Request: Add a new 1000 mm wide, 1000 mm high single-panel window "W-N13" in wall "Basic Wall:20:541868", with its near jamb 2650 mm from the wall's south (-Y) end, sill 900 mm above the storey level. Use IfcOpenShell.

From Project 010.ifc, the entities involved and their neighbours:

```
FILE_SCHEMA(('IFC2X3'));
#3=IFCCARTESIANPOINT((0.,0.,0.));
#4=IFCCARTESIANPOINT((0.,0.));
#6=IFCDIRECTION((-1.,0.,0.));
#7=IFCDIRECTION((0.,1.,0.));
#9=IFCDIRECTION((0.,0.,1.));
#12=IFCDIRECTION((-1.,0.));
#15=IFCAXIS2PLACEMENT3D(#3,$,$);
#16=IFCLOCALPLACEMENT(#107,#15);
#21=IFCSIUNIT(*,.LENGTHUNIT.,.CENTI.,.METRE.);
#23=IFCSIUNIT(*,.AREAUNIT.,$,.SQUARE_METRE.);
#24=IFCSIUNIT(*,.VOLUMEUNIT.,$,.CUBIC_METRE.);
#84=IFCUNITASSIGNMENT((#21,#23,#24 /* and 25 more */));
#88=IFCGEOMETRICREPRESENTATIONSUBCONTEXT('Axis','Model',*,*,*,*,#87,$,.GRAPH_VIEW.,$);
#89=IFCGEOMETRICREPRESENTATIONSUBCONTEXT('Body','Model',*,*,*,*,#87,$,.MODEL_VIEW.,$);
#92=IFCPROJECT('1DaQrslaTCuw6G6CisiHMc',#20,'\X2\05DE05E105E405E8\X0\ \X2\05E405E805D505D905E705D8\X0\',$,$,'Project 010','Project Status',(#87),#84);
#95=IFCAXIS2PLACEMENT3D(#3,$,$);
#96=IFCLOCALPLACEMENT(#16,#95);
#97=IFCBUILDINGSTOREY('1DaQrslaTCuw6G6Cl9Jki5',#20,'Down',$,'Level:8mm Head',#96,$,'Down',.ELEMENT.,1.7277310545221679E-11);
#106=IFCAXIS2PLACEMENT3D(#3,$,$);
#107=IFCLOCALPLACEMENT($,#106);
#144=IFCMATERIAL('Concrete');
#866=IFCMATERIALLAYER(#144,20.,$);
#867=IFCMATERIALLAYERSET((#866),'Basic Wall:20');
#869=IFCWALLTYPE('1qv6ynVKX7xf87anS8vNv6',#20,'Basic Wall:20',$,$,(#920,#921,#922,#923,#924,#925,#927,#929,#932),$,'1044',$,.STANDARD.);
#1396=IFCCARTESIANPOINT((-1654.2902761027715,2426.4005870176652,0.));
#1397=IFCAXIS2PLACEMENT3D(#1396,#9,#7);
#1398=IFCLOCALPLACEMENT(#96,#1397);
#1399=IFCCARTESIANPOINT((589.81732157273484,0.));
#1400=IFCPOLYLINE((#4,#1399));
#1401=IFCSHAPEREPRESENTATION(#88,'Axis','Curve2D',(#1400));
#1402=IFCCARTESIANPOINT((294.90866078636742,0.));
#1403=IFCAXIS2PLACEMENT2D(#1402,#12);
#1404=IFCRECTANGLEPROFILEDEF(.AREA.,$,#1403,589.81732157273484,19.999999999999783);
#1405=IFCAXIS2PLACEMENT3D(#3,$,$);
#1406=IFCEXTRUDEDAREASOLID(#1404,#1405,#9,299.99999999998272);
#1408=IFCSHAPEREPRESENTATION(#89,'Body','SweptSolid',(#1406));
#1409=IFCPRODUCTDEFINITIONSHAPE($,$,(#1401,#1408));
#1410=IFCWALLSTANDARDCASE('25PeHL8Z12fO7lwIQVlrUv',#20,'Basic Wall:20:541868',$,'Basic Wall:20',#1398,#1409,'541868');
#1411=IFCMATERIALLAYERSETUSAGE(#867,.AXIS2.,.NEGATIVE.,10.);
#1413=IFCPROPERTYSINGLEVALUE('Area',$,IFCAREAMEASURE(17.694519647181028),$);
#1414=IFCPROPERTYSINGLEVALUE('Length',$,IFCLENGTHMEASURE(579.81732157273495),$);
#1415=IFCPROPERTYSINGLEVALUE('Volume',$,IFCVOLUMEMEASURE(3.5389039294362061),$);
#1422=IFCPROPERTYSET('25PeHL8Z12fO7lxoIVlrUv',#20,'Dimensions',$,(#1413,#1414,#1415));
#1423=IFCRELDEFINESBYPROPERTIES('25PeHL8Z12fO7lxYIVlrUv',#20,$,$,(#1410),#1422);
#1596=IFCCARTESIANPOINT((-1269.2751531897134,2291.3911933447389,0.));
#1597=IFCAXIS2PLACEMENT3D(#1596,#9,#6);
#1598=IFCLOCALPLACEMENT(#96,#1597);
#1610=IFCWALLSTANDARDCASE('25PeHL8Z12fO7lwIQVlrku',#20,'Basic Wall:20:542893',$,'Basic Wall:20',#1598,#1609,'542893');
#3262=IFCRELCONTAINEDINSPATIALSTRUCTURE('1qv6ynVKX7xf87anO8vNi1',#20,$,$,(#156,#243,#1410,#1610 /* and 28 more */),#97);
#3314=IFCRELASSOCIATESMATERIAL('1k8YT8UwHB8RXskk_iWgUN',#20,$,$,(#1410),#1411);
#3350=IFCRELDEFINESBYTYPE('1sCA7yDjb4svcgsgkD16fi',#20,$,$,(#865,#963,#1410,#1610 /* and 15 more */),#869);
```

```python
import numpy as np
import ifcopenshell
import ifcopenshell.api.feature
import ifcopenshell.api.geometry
import ifcopenshell.api.pset
import ifcopenshell.api.root
import ifcopenshell.api.spatial
import ifcopenshell.api.type
import ifcopenshell.geom
import ifcopenshell.util.element
import ifcopenshell.util.placement
import ifcopenshell.util.representation
import ifcopenshell.util.shape
import ifcopenshell.util.unit

model = ifcopenshell.open("Project 010.ifc")
unit_scale = ifcopenshell.util.unit.calculate_unit_scale(model)
area_scale = ifcopenshell.util.unit.calculate_unit_scale(model, "AREAUNIT")
volume_scale = ifcopenshell.util.unit.calculate_unit_scale(model, "VOLUMEUNIT")
settings = ifcopenshell.geom.settings()


def volume(element):
    """Net volume in cubic metres, openings subtracted."""
    shape = ifcopenshell.geom.create_shape(settings, element)
    return ifcopenshell.util.shape.get_volume(shape.geometry)


wall = model.by_id(1410)
storey = ifcopenshell.util.element.get_container(wall, ifc_class="IfcBuildingStorey")
context = ifcopenshell.util.representation.get_context(model, "Model", "Body", "MODEL_VIEW")
before = volume(wall)

width, height, from_end, sill = 1, 1, 2.65, 0.9  # metres

# The wall runs along its own X axis, and the end named is its -X end.
wall_shape = ifcopenshell.geom.create_shape(settings, wall)
x, y, z = ifcopenshell.util.shape.get_vertices(wall_shape.geometry).T
start = x.min() + from_end
face, thickness = float(y.min()), float(y.max() - y.min())
wall_matrix = ifcopenshell.util.placement.get_local_placement(wall.ObjectPlacement)
level = ifcopenshell.util.placement.get_local_placement(storey.ObjectPlacement)[2, 3]


def in_wall(x, y):
    """Placement at x, y metres in the wall's axes, at sill height."""
    matrix = wall_matrix.copy()
    matrix[:, 3] = wall_matrix @ np.array([x / unit_scale, y / unit_scale, 0.0, 1.0])
    matrix[2, 3] = level + sill / unit_scale
    return matrix


# Opening: a box that overshoots both wall faces by 50 mm.
opening = ifcopenshell.api.root.create_entity(model, ifc_class="IfcOpeningElement")
box = ifcopenshell.api.geometry.add_wall_representation(
    model, context=context, length=width, height=height, thickness=thickness + 0.1
)
ifcopenshell.api.geometry.assign_representation(model, product=opening, representation=box)
ifcopenshell.api.geometry.edit_object_placement(model, product=opening, matrix=in_wall(start, face - 0.05), is_si=False)
ifcopenshell.api.feature.add_feature(model, feature=opening, element=wall)

window = ifcopenshell.api.root.create_entity(model, ifc_class="IfcWindow", name="W-N13")
window.OverallWidth, window.OverallHeight = width / unit_scale, height / unit_scale
body = ifcopenshell.api.geometry.add_window_representation(
    model,
    context=context,
    overall_width=window.OverallWidth,
    overall_height=window.OverallHeight,
    partition_type="SINGLE_PANEL",
)
ifcopenshell.api.geometry.assign_representation(model, product=window, representation=body)
ifcopenshell.api.spatial.assign_container(model, products=[window], relating_structure=storey)
fills = ifcopenshell.api.feature.add_filling(model, opening=opening, element=window)
fills.OwnerHistory = window.OwnerHistory  # required in IFC2X3

# IFC2X3 keeps the operation on the window style.
style = ifcopenshell.api.root.create_entity(model, ifc_class="IfcWindowStyle", name="W-N13")
style.OperationType, style.ConstructionType = "SINGLE_PANEL", "NOTDEFINED"
style.ParameterTakesPrecedence = style.Sizeable = False
ifcopenshell.api.type.assign_type(model, related_objects=[window], relating_type=style)

# Centre the window in the wall's thickness.
ifcopenshell.api.geometry.edit_object_placement(model, product=window, matrix=in_wall(start, face), is_si=False)
window_shape = ifcopenshell.geom.create_shape(settings, window)
depth = ifcopenshell.util.shape.get_vertices(window_shape.geometry)[:, 1]
offset = face + thickness / 2 - (depth.min() + depth.max()) / 2
ifcopenshell.api.geometry.edit_object_placement(model, product=window, matrix=in_wall(start, offset), is_si=False)

after = volume(wall)

# Update the wall's stored quantities.
pset = model.by_id(ifcopenshell.util.element.get_pset(wall, "Dimensions", should_inherit=False)["id"])
ifcopenshell.api.pset.edit_pset(model, pset=pset, properties={
    "Area": model.create_entity("IfcAreaMeasure", after / thickness / area_scale),
    "Volume": model.create_entity("IfcVolumeMeasure", after / volume_scale),
})

print(f"wall volume {before:.3f} -> {after:.3f} m3")

model.write("Project 010_v2.ifc")
```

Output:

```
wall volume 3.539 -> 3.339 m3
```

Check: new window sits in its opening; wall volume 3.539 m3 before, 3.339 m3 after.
